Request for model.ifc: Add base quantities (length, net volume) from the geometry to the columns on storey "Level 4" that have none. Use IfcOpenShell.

First a look at what the model holds.

```python
import ifcopenshell
import ifcopenshell.util.element
import ifcopenshell.util.unit

model = ifcopenshell.open("model.ifc")
print(model.schema)
for unit_type in ("LENGTHUNIT", "AREAUNIT", "VOLUMEUNIT"):
    print(unit_type, ifcopenshell.util.unit.calculate_unit_scale(model, unit_type))
storey = next(s for s in model.by_type("IfcBuildingStorey") if s.Name == "Level 4")
columns = [e for e in ifcopenshell.util.element.get_decomposition(storey) if e.is_a("IfcColumn")]
for e in sorted(columns, key=lambda e: e.id()):
    print(e.id(), e.is_a(), e.Name, list(ifcopenshell.util.element.get_psets(e, qtos_only=True)), sep=" | ")
```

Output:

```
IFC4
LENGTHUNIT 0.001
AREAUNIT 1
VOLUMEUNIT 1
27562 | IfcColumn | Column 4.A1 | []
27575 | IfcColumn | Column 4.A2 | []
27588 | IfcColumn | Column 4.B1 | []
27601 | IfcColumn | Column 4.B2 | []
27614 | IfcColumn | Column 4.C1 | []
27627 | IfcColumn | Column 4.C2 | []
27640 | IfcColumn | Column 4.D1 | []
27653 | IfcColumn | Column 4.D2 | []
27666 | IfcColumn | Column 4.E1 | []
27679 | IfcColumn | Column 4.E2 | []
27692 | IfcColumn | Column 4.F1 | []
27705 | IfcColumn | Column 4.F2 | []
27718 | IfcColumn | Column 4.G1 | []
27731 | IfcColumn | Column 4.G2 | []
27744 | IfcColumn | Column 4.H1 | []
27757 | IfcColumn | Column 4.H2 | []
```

```python
import ifcopenshell
import ifcopenshell.api.pset
import ifcopenshell.geom
import ifcopenshell.util.element
import ifcopenshell.util.shape
import ifcopenshell.util.unit

model = ifcopenshell.open("model.ifc")
unit_scale = ifcopenshell.util.unit.calculate_unit_scale(model)
volume_scale = ifcopenshell.util.unit.calculate_unit_scale(model, "VOLUMEUNIT")
settings = ifcopenshell.geom.settings()

storey = next(s for s in model.by_type("IfcBuildingStorey") if s.Name == "Level 4")
columns = [e for e in ifcopenshell.util.element.get_decomposition(storey) if e.is_a("IfcColumn")]

for e in sorted(columns, key=lambda e: e.id()):
    if ifcopenshell.util.element.get_psets(e, qtos_only=True, should_inherit=False):
        continue
    # Geometry comes back in metres, in the element's own axes.
    shape = ifcopenshell.geom.create_shape(settings, e)
    values = {
        "Length": ifcopenshell.util.shape.get_z(shape.geometry) / unit_scale,
        "NetVolume": ifcopenshell.util.shape.get_volume(shape.geometry) / volume_scale,
    }
    qto = ifcopenshell.api.pset.add_qto(model, product=e, name="Qto_ColumnBaseQuantities")
    ifcopenshell.api.pset.edit_qto(model, qto=qto, properties=values)
    print(e.id(), {k: round(v, 3) for k, v in values.items()})

model.write("model_v2.ifc")
```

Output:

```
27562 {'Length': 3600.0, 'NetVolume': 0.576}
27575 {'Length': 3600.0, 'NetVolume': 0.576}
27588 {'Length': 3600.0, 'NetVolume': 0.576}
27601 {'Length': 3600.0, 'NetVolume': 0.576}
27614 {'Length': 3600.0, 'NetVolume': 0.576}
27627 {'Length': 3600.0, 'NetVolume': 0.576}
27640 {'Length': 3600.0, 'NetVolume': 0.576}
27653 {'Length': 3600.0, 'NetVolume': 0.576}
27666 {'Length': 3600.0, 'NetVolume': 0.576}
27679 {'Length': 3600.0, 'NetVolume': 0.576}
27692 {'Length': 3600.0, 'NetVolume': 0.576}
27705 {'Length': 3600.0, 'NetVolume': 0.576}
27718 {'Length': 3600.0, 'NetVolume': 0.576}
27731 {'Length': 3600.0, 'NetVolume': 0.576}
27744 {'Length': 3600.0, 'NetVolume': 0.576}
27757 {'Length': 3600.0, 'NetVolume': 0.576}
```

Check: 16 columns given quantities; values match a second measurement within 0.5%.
